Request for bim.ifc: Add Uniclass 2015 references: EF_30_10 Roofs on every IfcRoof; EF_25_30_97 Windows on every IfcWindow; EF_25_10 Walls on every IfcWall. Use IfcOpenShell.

First a look at what the model holds.

```python
import ifcopenshell

model = ifcopenshell.open("bim.ifc")
print(model.schema)
print("classifications:", [c.Name for c in model.by_type("IfcClassification")])
for ifc_class in ("IfcDoor", "IfcRoof", "IfcStair", "IfcWall", "IfcWindow"):
    print(ifc_class, len(model.by_type(ifc_class)))
```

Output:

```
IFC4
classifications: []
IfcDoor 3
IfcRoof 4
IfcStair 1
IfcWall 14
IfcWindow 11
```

```python
import ifcopenshell
import ifcopenshell.api.classification

model = ifcopenshell.open("bim.ifc")

system = ifcopenshell.api.classification.add_classification(model, classification="Uniclass 2015")

codes = {
    "IfcRoof": ("EF_30_10", "Roofs"),
    "IfcWindow": ("EF_25_30_97", "Windows"),
    "IfcWall": ("EF_25_10", "Walls"),
}
for ifc_class, (code, name) in codes.items():
    products = model.by_type(ifc_class)
    ifcopenshell.api.classification.add_reference(
        model, products=products, classification=system, identification=code, name=name
    )
    print(code, len(products))

model.write("bim_edited.ifc")
```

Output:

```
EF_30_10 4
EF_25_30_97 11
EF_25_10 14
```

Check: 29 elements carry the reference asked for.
